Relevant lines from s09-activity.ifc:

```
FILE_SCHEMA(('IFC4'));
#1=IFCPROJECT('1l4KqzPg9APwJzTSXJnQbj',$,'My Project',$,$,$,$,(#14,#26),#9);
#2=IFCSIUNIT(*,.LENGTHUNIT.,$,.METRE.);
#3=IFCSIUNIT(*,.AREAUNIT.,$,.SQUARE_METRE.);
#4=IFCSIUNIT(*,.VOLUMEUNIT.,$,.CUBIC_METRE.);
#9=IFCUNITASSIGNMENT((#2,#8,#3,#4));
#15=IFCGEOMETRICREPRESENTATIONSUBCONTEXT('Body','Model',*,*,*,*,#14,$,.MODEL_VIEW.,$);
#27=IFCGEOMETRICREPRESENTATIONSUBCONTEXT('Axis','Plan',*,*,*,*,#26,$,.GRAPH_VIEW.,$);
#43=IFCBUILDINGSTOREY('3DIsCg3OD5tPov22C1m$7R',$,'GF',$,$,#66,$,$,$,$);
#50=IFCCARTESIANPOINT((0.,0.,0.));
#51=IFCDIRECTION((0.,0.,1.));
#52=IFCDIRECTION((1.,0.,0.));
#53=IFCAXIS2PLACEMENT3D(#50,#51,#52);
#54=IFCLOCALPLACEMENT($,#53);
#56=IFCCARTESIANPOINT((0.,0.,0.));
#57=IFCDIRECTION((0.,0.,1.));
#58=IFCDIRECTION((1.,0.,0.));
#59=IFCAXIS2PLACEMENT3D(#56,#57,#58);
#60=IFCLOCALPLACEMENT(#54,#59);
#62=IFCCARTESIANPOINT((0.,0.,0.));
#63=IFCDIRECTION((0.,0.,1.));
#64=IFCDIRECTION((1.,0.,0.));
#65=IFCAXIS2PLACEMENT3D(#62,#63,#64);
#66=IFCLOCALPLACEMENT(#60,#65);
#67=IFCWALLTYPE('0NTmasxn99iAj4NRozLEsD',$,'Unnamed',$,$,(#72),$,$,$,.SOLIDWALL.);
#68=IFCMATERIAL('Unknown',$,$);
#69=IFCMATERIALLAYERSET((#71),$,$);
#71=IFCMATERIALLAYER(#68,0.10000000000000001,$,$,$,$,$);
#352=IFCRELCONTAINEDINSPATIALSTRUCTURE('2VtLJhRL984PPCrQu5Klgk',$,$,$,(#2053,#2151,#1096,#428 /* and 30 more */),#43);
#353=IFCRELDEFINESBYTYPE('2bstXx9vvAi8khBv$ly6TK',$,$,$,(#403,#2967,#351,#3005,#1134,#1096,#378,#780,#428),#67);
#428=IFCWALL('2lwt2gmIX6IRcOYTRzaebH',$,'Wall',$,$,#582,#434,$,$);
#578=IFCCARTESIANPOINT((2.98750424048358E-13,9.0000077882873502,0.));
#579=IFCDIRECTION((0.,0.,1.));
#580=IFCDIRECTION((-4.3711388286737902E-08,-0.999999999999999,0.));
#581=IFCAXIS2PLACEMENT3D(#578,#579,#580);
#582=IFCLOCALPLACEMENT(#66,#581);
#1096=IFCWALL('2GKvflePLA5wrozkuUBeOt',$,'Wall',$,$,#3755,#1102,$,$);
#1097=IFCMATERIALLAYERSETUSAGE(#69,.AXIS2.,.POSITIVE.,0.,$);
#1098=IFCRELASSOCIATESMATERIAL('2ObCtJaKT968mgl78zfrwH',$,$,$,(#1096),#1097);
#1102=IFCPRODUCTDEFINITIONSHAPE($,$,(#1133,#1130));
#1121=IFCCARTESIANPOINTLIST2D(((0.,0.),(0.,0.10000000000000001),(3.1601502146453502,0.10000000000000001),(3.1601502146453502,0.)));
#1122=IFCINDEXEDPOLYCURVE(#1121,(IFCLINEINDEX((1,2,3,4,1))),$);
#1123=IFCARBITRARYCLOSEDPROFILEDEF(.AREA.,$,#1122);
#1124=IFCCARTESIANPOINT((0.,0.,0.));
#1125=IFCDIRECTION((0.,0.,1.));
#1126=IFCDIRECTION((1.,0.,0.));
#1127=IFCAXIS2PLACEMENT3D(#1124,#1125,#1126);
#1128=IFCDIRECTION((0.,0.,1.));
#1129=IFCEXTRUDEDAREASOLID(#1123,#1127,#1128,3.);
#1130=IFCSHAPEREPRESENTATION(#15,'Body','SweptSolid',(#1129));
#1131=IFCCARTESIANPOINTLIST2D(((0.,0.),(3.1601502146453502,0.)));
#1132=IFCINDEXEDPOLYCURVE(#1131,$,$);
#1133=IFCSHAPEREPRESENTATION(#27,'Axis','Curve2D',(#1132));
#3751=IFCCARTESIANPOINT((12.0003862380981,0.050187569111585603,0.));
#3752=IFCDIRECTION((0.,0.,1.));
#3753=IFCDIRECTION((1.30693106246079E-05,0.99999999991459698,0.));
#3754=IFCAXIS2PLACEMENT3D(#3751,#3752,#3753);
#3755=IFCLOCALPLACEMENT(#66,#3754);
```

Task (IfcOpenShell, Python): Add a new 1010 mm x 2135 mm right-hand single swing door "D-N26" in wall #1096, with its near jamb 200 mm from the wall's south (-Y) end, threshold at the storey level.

```python
import numpy as np
import ifcopenshell
import ifcopenshell.api.feature
import ifcopenshell.api.geometry
import ifcopenshell.api.root
import ifcopenshell.api.spatial
import ifcopenshell.geom
import ifcopenshell.util.element
import ifcopenshell.util.placement
import ifcopenshell.util.representation
import ifcopenshell.util.shape
import ifcopenshell.util.unit

model = ifcopenshell.open("s09-activity.ifc")
unit_scale = ifcopenshell.util.unit.calculate_unit_scale(model)
settings = ifcopenshell.geom.settings()


def volume(element):
    """Net volume in cubic metres, openings subtracted."""
    shape = ifcopenshell.geom.create_shape(settings, element)
    return ifcopenshell.util.shape.get_volume(shape.geometry)


wall = model.by_guid("2GKvflePLA5wrozkuUBeOt")
storey = ifcopenshell.util.element.get_container(wall, ifc_class="IfcBuildingStorey")
context = ifcopenshell.util.representation.get_context(model, "Model", "Body", "MODEL_VIEW")
before = volume(wall)

width, height, from_end, sill = 1.01, 2.135, 0.2, 0.0  # metres

# The wall runs along its own X axis, and the end named is its -X end.
wall_shape = ifcopenshell.geom.create_shape(settings, wall)
x, y, z = ifcopenshell.util.shape.get_vertices(wall_shape.geometry).T
start = x.min() + from_end
face, thickness = float(y.min()), float(y.max() - y.min())
wall_matrix = ifcopenshell.util.placement.get_local_placement(wall.ObjectPlacement)
level = ifcopenshell.util.placement.get_local_placement(storey.ObjectPlacement)[2, 3]


def in_wall(x, y):
    """Placement at x, y metres in the wall's axes, at sill height."""
    matrix = wall_matrix.copy()
    matrix[:, 3] = wall_matrix @ np.array([x / unit_scale, y / unit_scale, 0.0, 1.0])
    matrix[2, 3] = level + sill / unit_scale
    return matrix


# Opening: a box that overshoots both wall faces by 50 mm.
opening = ifcopenshell.api.root.create_entity(model, ifc_class="IfcOpeningElement", predefined_type="OPENING")
box = ifcopenshell.api.geometry.add_wall_representation(
    model, context=context, length=width, height=height, thickness=thickness + 0.1
)
ifcopenshell.api.geometry.assign_representation(model, product=opening, representation=box)
ifcopenshell.api.geometry.edit_object_placement(model, product=opening, matrix=in_wall(start, face - 0.05), is_si=False)
ifcopenshell.api.feature.add_feature(model, feature=opening, element=wall)

door = ifcopenshell.api.root.create_entity(model, ifc_class="IfcDoor", name="D-N26", predefined_type="DOOR")
door.OverallWidth, door.OverallHeight = width / unit_scale, height / unit_scale
door.OperationType = "SINGLE_SWING_RIGHT"
body = ifcopenshell.api.geometry.add_door_representation(
    model,
    context=context,
    overall_width=door.OverallWidth,
    overall_height=door.OverallHeight,
    operation_type="SINGLE_SWING_RIGHT",
    lining_properties={"LiningDepth": thickness / unit_scale, "ThresholdDepth": thickness / unit_scale},
)
ifcopenshell.api.geometry.assign_representation(model, product=door, representation=body)
ifcopenshell.api.spatial.assign_container(model, products=[door], relating_structure=storey)
ifcopenshell.api.feature.add_filling(model, opening=opening, element=door)

# The lining spans the wall, so the door starts at the wall face.
ifcopenshell.api.geometry.edit_object_placement(model, product=door, matrix=in_wall(start, face), is_si=False)

after = volume(wall)

print(f"wall volume {before:.3f} -> {after:.3f} m3")

model.write("s09-activity_updated.ifc")
```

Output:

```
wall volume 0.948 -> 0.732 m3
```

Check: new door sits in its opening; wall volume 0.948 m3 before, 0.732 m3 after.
